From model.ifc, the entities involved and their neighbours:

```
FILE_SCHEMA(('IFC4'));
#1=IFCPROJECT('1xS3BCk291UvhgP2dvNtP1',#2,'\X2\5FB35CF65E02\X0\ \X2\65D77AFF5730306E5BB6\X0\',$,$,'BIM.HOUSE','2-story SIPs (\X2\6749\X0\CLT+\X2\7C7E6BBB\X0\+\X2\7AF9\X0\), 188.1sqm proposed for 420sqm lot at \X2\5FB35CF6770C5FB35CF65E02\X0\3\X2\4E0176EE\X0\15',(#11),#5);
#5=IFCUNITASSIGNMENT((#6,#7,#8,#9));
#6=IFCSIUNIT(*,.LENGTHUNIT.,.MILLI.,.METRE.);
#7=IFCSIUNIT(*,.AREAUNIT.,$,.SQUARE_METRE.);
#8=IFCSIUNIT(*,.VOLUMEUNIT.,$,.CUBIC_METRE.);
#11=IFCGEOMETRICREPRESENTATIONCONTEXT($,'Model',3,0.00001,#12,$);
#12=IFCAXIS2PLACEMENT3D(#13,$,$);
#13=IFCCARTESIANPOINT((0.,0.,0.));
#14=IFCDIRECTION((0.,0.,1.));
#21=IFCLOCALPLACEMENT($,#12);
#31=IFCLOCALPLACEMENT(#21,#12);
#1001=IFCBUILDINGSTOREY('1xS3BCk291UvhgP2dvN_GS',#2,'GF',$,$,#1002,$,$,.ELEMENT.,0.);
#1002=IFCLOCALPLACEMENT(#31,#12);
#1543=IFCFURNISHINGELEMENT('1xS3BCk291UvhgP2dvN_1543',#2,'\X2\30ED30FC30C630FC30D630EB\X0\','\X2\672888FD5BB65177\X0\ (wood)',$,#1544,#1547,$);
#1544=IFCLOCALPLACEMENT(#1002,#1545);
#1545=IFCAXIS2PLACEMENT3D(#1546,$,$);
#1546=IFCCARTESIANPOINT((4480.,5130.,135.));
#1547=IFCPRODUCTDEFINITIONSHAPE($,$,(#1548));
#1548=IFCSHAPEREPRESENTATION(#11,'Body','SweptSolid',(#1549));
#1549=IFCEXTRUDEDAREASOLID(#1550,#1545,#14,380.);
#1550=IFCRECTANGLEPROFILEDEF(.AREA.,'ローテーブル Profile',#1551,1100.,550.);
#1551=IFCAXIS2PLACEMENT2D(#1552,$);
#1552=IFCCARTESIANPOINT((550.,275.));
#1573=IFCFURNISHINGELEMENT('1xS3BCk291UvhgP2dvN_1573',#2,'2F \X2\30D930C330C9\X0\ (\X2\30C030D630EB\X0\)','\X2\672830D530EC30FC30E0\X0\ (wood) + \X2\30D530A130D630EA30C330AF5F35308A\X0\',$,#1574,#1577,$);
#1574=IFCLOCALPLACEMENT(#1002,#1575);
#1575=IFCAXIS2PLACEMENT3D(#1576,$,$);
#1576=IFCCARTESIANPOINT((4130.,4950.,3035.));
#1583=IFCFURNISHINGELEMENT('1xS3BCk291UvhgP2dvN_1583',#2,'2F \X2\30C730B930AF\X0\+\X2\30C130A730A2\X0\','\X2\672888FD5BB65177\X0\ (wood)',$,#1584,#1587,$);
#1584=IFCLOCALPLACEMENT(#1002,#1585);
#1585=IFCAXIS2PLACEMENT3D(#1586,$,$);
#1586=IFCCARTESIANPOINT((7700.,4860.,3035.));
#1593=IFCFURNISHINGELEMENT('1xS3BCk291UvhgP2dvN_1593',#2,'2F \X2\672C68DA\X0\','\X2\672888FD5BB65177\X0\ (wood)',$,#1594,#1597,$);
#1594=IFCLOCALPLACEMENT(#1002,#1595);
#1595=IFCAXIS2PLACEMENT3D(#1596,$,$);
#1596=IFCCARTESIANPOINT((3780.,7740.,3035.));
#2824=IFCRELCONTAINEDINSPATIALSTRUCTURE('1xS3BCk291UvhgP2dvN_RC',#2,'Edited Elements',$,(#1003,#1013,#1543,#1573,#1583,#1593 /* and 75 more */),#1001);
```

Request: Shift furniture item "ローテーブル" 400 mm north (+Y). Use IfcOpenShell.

```python
import ifcopenshell
import ifcopenshell.api.geometry
import ifcopenshell.util.placement

model = ifcopenshell.open("model.ifc")

item = model.by_id(1543)
matrix = ifcopenshell.util.placement.get_local_placement(item.ObjectPlacement)
matrix[1, 3] += 400.0
ifcopenshell.api.geometry.edit_object_placement(model, product=item, matrix=matrix, is_si=False)

print(ifcopenshell.util.placement.get_local_placement(item.ObjectPlacement).round(3) + 0.0)

model.write("model_v2.ifc")
```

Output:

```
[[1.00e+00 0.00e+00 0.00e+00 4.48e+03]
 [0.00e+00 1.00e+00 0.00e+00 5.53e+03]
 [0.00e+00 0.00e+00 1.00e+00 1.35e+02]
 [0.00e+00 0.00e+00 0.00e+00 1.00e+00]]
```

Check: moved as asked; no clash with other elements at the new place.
